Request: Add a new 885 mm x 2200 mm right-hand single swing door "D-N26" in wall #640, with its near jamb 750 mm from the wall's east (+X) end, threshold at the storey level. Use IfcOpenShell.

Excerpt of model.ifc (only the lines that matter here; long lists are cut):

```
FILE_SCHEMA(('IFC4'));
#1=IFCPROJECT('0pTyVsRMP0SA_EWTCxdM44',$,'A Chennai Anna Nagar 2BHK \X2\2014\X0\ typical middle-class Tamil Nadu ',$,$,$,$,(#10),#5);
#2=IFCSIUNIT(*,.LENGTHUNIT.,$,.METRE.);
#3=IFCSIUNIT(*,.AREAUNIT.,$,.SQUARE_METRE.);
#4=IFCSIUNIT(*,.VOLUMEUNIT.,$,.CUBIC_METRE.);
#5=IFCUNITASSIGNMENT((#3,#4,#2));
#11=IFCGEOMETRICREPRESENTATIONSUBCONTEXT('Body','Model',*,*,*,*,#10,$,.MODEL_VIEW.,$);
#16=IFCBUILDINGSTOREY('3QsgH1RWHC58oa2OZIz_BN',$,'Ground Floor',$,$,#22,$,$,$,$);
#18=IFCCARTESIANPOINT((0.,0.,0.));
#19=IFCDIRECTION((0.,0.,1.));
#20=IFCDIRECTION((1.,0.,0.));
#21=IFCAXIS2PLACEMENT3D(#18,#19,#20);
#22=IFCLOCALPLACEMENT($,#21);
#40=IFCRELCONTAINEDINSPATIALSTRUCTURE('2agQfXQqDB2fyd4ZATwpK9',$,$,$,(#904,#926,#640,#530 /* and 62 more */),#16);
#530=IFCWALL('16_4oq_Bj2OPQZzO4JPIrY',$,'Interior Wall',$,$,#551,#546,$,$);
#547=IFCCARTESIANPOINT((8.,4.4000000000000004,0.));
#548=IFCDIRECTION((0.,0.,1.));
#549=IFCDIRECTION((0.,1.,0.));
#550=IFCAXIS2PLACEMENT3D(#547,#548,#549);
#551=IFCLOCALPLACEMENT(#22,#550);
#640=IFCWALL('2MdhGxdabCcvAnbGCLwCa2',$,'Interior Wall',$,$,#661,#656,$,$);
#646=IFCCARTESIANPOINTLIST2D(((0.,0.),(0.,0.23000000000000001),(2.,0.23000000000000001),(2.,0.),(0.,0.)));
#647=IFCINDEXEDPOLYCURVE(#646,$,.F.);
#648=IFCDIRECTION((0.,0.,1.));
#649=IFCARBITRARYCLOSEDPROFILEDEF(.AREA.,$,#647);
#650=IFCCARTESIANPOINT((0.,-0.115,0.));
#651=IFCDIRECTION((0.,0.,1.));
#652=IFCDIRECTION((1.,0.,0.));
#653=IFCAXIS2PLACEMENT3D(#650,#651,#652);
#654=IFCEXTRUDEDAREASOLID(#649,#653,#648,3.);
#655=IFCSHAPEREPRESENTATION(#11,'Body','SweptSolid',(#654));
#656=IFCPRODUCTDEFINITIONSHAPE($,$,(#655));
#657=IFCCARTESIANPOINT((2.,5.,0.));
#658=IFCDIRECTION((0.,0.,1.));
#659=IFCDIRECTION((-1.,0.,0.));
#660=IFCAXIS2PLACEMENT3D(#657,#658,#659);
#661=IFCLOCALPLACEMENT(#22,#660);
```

```python
import numpy as np
import ifcopenshell
import ifcopenshell.api.feature
import ifcopenshell.api.geometry
import ifcopenshell.api.root
import ifcopenshell.api.spatial
import ifcopenshell.geom
import ifcopenshell.util.element
import ifcopenshell.util.placement
import ifcopenshell.util.representation
import ifcopenshell.util.shape
import ifcopenshell.util.unit

model = ifcopenshell.open("model.ifc")
unit_scale = ifcopenshell.util.unit.calculate_unit_scale(model)
settings = ifcopenshell.geom.settings()


def volume(element):
    """Net volume in cubic metres, openings subtracted."""
    shape = ifcopenshell.geom.create_shape(settings, element)
    return ifcopenshell.util.shape.get_volume(shape.geometry)


wall = model.by_guid("2MdhGxdabCcvAnbGCLwCa2")
storey = ifcopenshell.util.element.get_container(wall, ifc_class="IfcBuildingStorey")
context = ifcopenshell.util.representation.get_context(model, "Model", "Body", "MODEL_VIEW")
before = volume(wall)

width, height, from_end, sill = 0.885, 2.2, 0.75, 0.0  # metres

# The wall runs along its own X axis, and the end named is its -X end.
wall_shape = ifcopenshell.geom.create_shape(settings, wall)
x, y, z = ifcopenshell.util.shape.get_vertices(wall_shape.geometry).T
start = x.min() + from_end
face, thickness = float(y.min()), float(y.max() - y.min())
wall_matrix = ifcopenshell.util.placement.get_local_placement(wall.ObjectPlacement)
level = ifcopenshell.util.placement.get_local_placement(storey.ObjectPlacement)[2, 3]


def in_wall(x, y):
    """Placement at x, y metres in the wall's axes, at sill height."""
    matrix = wall_matrix.copy()
    matrix[:, 3] = wall_matrix @ np.array([x / unit_scale, y / unit_scale, 0.0, 1.0])
    matrix[2, 3] = level + sill / unit_scale
    return matrix


# Opening: a box that overshoots both wall faces by 50 mm.
opening = ifcopenshell.api.root.create_entity(model, ifc_class="IfcOpeningElement", predefined_type="OPENING")
box = ifcopenshell.api.geometry.add_wall_representation(
    model, context=context, length=width, height=height, thickness=thickness + 0.1
)
ifcopenshell.api.geometry.assign_representation(model, product=opening, representation=box)
ifcopenshell.api.geometry.edit_object_placement(model, product=opening, matrix=in_wall(start, face - 0.05), is_si=False)
ifcopenshell.api.feature.add_feature(model, feature=opening, element=wall)

door = ifcopenshell.api.root.create_entity(model, ifc_class="IfcDoor", name="D-N26", predefined_type="DOOR")
door.OverallWidth, door.OverallHeight = width / unit_scale, height / unit_scale
door.OperationType = "SINGLE_SWING_RIGHT"
body = ifcopenshell.api.geometry.add_door_representation(
    model,
    context=context,
    overall_width=door.OverallWidth,
    overall_height=door.OverallHeight,
    operation_type="SINGLE_SWING_RIGHT",
    lining_properties={"LiningDepth": thickness / unit_scale, "ThresholdDepth": thickness / unit_scale},
)
ifcopenshell.api.geometry.assign_representation(model, product=door, representation=body)
ifcopenshell.api.spatial.assign_container(model, products=[door], relating_structure=storey)
ifcopenshell.api.feature.add_filling(model, opening=opening, element=door)

# The lining spans the wall, so the door starts at the wall face.
ifcopenshell.api.geometry.edit_object_placement(model, product=door, matrix=in_wall(start, face), is_si=False)

after = volume(wall)

print(f"wall volume {before:.3f} -> {after:.3f} m3")

model.write("model_rev.ifc")
```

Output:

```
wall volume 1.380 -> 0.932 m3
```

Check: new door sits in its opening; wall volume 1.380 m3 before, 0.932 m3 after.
